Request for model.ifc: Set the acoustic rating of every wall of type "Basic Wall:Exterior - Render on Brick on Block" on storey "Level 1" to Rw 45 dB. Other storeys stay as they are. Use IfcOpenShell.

First a look at what the model holds.

```python
import ifcopenshell
import ifcopenshell.util.element

model = ifcopenshell.open("model.ifc")
print(model.schema)
storey = next(s for s in model.by_type("IfcBuildingStorey") if s.Name == "Level 1")
walls = [e for e in ifcopenshell.util.element.get_decomposition(storey) if e.is_a("IfcWall")]
seen = {}
for e in walls:
    element_type = ifcopenshell.util.element.get_type(e)
    key = (element_type.Name if element_type != e and element_type else None, ifcopenshell.util.element.get_pset(e, "Pset_WallCommon", "AcousticRating"))
    seen[key] = seen.get(key, 0) + 1
for (name, value), count in sorted(seen.items(), key=str):
    print(count, "x", name, "|", value)
```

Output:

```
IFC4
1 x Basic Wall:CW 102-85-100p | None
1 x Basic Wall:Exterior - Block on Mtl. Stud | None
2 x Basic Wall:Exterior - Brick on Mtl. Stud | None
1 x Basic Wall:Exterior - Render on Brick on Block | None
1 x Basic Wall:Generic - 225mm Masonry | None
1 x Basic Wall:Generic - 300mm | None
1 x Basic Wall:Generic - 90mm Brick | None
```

```python
import ifcopenshell
import ifcopenshell.api.pset
import ifcopenshell.util.element

model = ifcopenshell.open("model.ifc")

storey = next(s for s in model.by_type("IfcBuildingStorey") if s.Name == "Level 1")
walls = [e for e in ifcopenshell.util.element.get_decomposition(storey) if e.is_a("IfcWall")]

count = 0
for e in walls:
    element_type = ifcopenshell.util.element.get_type(e)
    if element_type in (None, e) or element_type.Name != "Basic Wall:Exterior - Render on Brick on Block":
        continue
    # add_pset returns the element's existing set when there is one.
    pset = ifcopenshell.api.pset.add_pset(model, product=e, name="Pset_WallCommon")
    ifcopenshell.api.pset.edit_pset(model, pset=pset, properties={"AcousticRating": "Rw 45 dB"})
    count += 1

print(count, "walls updated")

model.write("model_rev.ifc")
```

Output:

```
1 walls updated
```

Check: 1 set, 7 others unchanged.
